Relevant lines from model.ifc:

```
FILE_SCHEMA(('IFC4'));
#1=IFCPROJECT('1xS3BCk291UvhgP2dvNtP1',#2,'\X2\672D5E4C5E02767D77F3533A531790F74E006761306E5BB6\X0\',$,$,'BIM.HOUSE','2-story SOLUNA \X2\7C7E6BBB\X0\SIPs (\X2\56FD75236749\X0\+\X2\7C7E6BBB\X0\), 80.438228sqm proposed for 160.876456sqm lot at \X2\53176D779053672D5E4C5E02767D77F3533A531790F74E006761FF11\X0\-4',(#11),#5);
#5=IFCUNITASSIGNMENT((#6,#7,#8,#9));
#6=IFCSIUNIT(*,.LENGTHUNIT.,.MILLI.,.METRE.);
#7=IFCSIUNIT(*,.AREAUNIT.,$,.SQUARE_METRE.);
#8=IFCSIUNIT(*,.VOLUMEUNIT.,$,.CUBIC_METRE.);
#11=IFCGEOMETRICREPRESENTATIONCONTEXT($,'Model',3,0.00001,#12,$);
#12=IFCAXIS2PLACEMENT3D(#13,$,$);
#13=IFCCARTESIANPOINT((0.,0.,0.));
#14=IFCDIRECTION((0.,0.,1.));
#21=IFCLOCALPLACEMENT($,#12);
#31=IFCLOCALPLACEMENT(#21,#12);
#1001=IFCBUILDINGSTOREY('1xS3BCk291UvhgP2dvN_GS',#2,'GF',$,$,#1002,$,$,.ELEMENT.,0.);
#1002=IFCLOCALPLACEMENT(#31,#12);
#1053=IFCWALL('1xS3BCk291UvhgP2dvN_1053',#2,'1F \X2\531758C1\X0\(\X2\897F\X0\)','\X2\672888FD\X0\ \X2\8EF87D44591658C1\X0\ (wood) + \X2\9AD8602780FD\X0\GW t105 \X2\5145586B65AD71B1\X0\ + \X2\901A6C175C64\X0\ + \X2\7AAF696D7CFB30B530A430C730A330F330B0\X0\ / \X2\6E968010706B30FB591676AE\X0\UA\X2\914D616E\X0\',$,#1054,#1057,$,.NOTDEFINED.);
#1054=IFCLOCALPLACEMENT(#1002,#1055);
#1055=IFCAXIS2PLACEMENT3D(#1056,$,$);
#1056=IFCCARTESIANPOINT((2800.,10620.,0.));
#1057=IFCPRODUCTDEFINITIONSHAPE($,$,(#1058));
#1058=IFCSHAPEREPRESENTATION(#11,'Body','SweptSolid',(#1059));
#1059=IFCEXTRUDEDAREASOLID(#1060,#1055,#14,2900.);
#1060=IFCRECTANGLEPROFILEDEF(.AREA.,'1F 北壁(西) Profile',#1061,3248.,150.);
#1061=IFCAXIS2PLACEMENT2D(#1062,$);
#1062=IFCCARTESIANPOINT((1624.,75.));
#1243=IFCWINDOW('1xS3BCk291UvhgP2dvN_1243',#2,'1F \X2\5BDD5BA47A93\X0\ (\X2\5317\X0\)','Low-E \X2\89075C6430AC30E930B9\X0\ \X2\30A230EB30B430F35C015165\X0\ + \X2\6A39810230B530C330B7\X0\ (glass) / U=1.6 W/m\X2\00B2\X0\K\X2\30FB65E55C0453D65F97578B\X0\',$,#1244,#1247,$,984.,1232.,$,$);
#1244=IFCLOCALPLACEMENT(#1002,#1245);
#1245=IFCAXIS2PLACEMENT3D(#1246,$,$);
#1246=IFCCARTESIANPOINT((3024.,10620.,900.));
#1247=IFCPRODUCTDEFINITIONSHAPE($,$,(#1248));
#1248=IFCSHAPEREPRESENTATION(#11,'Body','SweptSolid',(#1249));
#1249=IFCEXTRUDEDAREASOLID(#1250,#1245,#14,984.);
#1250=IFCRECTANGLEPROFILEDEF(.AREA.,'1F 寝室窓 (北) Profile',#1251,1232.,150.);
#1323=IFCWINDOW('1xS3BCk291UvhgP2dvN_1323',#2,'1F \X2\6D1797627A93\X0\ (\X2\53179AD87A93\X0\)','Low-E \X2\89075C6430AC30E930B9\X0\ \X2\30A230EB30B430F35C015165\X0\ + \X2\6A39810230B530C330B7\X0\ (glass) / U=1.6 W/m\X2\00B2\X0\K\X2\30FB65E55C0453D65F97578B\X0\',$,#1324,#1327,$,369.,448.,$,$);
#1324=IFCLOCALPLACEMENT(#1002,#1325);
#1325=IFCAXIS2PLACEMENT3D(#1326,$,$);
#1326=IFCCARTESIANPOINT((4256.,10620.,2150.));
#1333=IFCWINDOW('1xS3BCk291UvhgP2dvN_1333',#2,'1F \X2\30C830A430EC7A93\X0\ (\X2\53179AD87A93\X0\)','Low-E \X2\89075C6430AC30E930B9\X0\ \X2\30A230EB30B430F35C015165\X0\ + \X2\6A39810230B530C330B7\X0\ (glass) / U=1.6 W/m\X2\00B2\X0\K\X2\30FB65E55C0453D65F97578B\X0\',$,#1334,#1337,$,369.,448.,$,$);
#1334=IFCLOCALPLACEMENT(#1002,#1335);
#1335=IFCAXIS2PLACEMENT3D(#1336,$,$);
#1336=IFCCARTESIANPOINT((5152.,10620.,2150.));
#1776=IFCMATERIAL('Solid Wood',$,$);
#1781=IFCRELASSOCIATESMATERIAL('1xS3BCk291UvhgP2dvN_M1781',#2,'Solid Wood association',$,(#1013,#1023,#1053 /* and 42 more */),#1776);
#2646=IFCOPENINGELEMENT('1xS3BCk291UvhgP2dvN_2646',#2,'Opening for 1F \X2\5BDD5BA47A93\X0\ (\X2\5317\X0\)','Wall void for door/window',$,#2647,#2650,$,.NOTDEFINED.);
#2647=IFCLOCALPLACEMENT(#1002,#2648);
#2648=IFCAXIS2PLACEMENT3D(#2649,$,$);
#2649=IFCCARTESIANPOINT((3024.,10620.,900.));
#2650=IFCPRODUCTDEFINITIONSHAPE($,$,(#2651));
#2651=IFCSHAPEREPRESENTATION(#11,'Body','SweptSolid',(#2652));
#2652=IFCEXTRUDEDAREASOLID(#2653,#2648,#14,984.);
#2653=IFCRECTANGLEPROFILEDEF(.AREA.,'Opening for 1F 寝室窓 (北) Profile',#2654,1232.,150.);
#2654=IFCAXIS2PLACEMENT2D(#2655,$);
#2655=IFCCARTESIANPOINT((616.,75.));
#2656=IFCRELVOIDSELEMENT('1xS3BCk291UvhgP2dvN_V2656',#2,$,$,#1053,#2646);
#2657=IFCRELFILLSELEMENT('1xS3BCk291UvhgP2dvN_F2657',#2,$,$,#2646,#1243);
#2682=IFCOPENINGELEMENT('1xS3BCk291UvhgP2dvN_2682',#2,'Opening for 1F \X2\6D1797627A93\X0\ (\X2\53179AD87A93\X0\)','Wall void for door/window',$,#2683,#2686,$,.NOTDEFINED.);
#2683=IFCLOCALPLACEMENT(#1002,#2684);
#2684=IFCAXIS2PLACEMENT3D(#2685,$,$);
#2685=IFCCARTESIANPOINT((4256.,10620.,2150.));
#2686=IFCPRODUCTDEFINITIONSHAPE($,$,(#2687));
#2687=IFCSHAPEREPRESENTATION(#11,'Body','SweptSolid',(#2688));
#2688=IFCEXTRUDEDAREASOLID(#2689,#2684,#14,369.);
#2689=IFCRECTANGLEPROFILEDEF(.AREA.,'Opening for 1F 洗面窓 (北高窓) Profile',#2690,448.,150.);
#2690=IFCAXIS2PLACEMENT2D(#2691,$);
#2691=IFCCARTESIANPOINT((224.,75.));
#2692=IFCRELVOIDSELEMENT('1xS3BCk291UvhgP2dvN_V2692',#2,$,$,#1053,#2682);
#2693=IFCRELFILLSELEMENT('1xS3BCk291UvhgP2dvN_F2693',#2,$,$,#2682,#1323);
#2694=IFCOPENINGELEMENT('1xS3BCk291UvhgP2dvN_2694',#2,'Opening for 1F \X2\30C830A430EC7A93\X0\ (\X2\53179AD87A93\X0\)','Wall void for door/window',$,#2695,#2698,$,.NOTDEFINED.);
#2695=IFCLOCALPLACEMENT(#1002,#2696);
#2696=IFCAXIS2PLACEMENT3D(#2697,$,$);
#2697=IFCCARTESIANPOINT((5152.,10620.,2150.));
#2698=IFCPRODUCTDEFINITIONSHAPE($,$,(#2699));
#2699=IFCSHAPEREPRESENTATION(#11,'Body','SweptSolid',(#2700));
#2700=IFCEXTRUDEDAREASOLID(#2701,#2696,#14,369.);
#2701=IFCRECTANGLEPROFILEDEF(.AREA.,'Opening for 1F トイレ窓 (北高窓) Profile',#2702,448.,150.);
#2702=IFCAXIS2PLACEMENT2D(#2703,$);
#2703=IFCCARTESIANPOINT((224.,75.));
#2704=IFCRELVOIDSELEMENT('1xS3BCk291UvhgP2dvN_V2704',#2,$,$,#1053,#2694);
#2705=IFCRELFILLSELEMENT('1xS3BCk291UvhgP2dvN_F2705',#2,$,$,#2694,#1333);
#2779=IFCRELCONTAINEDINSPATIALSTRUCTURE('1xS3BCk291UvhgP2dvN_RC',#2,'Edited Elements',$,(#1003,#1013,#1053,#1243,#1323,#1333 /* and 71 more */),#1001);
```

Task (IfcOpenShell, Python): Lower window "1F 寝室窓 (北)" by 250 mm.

```python
import numpy as np
import ifcopenshell
import ifcopenshell.api.geometry
import ifcopenshell.util.placement
import ifcopenshell.util.unit

model = ifcopenshell.open("model.ifc")
unit_scale = ifcopenshell.util.unit.calculate_unit_scale(model)

window = model.by_id(1243)
opening = window.FillsVoids[0].RelatingOpeningElement
dz = -250.0

shift = np.array([0.0, 0.0, dz])
# The window is not placed relative to its opening, so move both.
for product in (opening, window):
    matrix = ifcopenshell.util.placement.get_local_placement(product.ObjectPlacement)
    matrix[:3, 3] += shift
    ifcopenshell.api.geometry.edit_object_placement(model, product=product, matrix=matrix, is_si=False)

print(f"moved by {dz * unit_scale:+.3f} m")

model.write("model_v2.ifc")
```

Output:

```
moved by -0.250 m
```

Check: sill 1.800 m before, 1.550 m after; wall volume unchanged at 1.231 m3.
